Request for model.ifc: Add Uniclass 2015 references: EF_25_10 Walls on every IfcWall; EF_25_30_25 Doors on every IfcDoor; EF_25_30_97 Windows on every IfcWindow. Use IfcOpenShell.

First a look at what the model holds.

```python
import ifcopenshell

model = ifcopenshell.open("model.ifc")
print(model.schema)
print("classifications:", [c.Name for c in model.by_type("IfcClassification")])
for ifc_class in ("IfcDoor", "IfcRoof", "IfcStair", "IfcWall", "IfcWindow"):
    print(ifc_class, len(model.by_type(ifc_class)))
```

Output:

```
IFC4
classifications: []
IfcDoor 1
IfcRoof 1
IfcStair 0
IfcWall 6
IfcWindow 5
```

```python
import ifcopenshell
import ifcopenshell.api.classification

model = ifcopenshell.open("model.ifc")

system = ifcopenshell.api.classification.add_classification(model, classification="Uniclass 2015")

codes = {
    "IfcWall": ("EF_25_10", "Walls"),
    "IfcDoor": ("EF_25_30_25", "Doors"),
    "IfcWindow": ("EF_25_30_97", "Windows"),
}
for ifc_class, (code, name) in codes.items():
    products = model.by_type(ifc_class)
    ifcopenshell.api.classification.add_reference(
        model, products=products, classification=system, identification=code, name=name
    )
    print(code, len(products))

model.write("model_updated.ifc")
```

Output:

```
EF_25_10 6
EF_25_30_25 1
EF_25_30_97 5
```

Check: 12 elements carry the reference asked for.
